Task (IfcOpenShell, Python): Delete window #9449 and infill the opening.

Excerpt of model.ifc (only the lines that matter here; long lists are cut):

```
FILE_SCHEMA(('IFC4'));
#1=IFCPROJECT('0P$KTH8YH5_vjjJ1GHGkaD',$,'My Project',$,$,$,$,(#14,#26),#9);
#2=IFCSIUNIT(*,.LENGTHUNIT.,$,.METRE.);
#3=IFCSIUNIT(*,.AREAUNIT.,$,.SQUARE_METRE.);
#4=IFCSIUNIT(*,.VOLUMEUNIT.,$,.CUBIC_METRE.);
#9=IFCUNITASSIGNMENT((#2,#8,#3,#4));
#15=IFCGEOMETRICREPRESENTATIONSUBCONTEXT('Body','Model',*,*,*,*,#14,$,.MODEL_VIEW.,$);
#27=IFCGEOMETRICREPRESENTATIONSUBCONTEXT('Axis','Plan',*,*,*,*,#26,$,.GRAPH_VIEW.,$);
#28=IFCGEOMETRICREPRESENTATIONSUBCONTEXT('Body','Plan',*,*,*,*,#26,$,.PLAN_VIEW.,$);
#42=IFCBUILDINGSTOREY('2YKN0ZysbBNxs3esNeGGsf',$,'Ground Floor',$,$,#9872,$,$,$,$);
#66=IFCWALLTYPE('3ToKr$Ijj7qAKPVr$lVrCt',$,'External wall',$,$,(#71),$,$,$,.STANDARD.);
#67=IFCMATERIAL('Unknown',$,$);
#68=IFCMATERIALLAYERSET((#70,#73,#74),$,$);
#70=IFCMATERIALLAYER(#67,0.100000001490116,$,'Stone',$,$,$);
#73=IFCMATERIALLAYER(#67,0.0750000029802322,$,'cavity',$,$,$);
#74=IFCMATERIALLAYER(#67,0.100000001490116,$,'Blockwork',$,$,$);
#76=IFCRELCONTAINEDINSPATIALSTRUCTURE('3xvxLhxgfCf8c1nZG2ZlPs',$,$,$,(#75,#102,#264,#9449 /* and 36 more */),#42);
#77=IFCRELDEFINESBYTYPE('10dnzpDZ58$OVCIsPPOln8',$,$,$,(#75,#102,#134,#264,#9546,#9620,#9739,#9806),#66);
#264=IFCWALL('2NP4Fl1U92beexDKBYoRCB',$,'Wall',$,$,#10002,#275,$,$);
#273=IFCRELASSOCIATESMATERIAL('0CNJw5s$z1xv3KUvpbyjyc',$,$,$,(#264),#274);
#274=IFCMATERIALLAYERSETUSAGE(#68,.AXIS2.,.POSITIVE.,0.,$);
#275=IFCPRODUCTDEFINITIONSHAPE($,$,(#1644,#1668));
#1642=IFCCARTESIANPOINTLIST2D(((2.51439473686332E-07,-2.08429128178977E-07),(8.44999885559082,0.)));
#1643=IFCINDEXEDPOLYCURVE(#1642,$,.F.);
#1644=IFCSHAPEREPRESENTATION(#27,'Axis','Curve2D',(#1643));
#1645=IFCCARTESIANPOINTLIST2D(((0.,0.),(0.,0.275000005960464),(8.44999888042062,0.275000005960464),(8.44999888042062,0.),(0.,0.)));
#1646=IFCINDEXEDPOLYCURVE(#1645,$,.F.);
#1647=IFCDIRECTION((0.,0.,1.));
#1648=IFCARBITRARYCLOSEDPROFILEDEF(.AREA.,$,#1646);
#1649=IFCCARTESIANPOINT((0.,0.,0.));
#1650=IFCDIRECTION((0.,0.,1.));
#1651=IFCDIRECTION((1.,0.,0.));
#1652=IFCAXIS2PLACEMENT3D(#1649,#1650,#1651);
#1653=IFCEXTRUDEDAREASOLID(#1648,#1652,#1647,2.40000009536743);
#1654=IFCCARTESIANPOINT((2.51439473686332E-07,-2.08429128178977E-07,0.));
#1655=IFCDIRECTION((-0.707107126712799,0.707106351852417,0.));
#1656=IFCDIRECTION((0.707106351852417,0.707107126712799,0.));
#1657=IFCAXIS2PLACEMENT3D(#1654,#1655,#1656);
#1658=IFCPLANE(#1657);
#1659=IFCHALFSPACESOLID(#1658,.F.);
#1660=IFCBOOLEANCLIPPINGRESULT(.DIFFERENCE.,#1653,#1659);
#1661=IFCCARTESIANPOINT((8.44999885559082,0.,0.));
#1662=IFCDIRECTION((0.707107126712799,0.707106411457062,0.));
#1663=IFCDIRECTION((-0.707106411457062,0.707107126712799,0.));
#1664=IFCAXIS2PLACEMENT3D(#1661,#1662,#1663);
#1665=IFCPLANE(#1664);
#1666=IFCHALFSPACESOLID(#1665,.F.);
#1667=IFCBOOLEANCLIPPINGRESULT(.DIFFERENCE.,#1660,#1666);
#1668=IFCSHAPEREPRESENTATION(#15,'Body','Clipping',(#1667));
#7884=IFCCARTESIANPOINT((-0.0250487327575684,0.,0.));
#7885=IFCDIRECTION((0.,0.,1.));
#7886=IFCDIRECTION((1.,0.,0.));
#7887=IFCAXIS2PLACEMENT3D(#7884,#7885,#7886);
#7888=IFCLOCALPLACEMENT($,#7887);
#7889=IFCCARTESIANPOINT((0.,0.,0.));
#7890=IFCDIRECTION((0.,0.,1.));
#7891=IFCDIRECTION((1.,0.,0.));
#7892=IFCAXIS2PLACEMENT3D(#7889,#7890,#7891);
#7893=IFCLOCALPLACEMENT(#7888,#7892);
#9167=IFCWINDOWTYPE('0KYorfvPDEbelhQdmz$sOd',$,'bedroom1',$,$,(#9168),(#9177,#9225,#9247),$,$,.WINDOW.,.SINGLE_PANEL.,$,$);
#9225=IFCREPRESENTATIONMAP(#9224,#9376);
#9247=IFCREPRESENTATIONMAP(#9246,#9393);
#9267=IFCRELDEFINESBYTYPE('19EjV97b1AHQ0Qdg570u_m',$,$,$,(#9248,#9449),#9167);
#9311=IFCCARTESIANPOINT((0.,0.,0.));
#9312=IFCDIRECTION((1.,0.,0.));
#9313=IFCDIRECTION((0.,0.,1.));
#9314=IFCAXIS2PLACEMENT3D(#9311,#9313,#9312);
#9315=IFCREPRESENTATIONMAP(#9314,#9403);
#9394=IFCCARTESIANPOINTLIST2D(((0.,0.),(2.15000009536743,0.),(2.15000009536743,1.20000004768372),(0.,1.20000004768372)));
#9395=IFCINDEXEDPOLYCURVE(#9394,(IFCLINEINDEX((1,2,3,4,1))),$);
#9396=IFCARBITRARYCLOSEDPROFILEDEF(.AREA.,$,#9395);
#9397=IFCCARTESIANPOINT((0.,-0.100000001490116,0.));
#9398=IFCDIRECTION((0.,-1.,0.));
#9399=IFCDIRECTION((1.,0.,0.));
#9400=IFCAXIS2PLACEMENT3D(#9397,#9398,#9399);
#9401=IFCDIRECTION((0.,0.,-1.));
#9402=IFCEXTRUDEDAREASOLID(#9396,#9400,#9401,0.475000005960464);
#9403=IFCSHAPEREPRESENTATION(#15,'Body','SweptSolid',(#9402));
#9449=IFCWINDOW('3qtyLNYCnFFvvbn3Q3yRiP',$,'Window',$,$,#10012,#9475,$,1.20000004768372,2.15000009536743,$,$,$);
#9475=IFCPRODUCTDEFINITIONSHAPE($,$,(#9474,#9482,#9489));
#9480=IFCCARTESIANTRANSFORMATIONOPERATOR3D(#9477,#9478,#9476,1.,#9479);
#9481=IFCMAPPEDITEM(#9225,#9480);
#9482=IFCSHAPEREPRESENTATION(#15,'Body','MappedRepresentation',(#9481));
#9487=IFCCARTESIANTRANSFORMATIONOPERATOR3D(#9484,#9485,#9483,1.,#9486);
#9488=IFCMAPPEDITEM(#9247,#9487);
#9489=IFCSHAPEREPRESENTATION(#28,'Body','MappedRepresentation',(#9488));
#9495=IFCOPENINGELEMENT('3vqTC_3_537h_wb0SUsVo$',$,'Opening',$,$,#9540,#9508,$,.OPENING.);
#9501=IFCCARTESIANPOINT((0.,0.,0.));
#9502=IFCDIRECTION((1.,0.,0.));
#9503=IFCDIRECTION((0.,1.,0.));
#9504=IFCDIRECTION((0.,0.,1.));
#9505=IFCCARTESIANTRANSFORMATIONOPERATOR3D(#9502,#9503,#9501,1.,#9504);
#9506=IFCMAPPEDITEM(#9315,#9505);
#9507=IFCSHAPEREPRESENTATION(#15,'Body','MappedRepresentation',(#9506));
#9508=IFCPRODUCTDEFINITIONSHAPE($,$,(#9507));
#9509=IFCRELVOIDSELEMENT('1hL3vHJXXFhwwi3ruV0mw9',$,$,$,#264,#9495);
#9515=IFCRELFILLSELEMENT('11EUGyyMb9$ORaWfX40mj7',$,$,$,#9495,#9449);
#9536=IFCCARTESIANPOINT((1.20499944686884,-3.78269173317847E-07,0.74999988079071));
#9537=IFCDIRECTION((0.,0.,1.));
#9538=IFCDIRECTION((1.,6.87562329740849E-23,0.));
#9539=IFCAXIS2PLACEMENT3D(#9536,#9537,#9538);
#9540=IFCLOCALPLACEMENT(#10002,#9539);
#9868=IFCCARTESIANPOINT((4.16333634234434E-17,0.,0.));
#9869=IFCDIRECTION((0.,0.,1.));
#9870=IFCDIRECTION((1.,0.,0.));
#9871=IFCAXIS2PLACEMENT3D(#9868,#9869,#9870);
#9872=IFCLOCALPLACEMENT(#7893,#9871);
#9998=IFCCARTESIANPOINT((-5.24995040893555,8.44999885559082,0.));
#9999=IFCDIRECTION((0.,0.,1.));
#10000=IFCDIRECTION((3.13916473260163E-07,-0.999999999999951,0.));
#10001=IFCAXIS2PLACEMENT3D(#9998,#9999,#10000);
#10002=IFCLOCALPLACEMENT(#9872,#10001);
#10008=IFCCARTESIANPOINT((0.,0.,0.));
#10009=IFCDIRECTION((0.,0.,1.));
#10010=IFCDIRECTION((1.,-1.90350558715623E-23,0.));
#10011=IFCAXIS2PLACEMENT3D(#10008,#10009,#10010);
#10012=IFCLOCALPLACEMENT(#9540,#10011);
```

```python
import ifcopenshell
import ifcopenshell.api.feature
import ifcopenshell.api.root
import ifcopenshell.geom
import ifcopenshell.util.shape

model = ifcopenshell.open("model.ifc")
settings = ifcopenshell.geom.settings()


def volume(element):
    """Net volume in cubic metres, openings subtracted."""
    shape = ifcopenshell.geom.create_shape(settings, element)
    return ifcopenshell.util.shape.get_volume(shape.geometry)


window = model.by_guid("3qtyLNYCnFFvvbn3Q3yRiP")
opening = window.FillsVoids[0].RelatingOpeningElement
wall = opening.VoidsElements[0].RelatingBuildingElement
before = volume(wall)

ifcopenshell.api.root.remove_product(model, product=window)
ifcopenshell.api.feature.remove_feature(model, feature=opening)

after = volume(wall)

print(f"wall volume {before:.3f} -> {after:.3f} m3")

model.write("model_v2.ifc")
```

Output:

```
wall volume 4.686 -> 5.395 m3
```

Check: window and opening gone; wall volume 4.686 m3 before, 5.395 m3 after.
